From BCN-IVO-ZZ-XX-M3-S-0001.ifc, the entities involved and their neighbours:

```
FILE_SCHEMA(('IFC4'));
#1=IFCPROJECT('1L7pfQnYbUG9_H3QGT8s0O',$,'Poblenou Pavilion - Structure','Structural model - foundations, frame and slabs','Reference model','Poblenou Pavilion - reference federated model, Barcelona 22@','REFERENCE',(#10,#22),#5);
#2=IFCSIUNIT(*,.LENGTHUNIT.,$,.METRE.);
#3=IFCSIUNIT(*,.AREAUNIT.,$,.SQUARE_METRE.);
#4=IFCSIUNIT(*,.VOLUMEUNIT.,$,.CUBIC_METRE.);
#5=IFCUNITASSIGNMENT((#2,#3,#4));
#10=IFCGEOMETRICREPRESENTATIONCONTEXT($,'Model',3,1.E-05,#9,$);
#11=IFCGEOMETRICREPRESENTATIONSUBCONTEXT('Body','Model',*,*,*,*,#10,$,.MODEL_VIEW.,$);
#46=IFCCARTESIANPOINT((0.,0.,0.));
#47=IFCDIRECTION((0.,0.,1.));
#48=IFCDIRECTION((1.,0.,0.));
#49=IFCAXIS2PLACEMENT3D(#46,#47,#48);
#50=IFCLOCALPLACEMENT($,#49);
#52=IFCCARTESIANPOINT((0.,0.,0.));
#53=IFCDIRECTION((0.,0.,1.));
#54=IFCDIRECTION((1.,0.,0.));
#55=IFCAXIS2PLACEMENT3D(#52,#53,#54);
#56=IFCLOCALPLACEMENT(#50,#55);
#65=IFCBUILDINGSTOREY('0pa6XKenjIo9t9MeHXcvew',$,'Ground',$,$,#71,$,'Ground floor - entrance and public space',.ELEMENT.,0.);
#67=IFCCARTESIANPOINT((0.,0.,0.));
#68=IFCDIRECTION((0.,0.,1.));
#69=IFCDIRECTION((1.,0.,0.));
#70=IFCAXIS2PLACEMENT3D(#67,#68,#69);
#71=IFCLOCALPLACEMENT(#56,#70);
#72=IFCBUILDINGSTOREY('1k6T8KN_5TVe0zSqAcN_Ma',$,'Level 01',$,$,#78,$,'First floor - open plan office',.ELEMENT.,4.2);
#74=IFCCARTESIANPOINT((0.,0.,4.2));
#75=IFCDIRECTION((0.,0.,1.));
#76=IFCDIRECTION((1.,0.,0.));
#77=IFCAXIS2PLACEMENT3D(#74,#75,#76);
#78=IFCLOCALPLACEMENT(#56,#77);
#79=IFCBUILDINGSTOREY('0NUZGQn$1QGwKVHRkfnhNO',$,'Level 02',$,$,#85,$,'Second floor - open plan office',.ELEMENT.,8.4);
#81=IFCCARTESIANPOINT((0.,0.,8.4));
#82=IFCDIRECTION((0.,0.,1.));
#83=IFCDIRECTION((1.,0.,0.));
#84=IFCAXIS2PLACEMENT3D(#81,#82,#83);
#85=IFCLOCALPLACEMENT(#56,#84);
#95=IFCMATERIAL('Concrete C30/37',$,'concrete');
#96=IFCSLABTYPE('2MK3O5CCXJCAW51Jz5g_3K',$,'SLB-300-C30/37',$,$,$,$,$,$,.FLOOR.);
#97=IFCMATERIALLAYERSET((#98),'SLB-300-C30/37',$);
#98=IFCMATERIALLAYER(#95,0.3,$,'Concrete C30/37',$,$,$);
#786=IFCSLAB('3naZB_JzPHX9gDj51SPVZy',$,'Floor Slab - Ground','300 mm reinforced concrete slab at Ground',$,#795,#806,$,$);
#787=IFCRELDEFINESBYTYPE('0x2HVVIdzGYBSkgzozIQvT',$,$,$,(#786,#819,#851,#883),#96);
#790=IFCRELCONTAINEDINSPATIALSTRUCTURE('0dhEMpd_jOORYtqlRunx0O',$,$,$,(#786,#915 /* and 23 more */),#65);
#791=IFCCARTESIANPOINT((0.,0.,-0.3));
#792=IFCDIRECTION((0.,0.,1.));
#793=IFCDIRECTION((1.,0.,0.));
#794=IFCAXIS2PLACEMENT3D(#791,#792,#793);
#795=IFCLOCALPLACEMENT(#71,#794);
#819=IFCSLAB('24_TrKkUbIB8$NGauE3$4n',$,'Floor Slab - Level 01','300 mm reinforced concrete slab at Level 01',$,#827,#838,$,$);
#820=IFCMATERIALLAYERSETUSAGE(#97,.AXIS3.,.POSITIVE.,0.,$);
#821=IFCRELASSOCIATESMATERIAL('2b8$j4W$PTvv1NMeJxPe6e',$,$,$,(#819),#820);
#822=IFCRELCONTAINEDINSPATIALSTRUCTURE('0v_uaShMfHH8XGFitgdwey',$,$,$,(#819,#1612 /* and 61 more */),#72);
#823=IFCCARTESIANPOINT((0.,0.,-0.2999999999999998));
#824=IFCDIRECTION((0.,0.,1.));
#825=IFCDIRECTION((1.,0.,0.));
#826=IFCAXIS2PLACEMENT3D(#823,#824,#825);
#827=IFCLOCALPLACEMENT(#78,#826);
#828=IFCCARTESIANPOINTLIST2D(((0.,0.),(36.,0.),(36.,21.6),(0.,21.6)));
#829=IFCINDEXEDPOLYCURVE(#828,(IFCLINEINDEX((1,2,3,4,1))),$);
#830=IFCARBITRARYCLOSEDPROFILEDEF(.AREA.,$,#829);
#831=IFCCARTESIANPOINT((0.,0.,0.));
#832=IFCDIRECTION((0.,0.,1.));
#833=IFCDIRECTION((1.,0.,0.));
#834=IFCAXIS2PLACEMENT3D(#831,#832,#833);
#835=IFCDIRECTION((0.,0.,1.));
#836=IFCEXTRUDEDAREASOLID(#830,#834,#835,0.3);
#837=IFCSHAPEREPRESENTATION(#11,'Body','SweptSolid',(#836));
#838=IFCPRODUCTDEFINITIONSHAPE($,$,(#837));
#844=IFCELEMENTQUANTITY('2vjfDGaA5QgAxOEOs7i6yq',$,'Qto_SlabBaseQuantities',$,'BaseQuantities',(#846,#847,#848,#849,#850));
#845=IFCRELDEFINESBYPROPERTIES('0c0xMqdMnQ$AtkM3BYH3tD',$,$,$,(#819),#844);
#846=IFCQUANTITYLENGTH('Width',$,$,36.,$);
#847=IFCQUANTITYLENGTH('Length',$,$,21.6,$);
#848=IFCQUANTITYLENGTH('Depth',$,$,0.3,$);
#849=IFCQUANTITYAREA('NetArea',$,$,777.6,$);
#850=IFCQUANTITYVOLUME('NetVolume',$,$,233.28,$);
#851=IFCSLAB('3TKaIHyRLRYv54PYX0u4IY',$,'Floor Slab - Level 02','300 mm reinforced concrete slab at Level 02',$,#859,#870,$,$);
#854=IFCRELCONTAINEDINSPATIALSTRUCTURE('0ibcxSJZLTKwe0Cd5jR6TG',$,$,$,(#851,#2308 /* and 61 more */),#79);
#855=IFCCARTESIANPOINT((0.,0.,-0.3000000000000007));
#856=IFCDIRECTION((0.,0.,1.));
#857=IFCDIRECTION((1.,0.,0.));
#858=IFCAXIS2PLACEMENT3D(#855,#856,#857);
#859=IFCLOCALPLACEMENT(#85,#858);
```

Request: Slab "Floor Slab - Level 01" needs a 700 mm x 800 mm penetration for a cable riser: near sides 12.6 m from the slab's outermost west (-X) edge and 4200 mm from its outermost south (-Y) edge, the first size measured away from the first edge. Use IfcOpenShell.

```python
import numpy as np
import ifcopenshell
import ifcopenshell.api.feature
import ifcopenshell.api.geometry
import ifcopenshell.api.pset
import ifcopenshell.api.root
import ifcopenshell.geom
import ifcopenshell.util.element
import ifcopenshell.util.placement
import ifcopenshell.util.representation
import ifcopenshell.util.shape
import ifcopenshell.util.unit

model = ifcopenshell.open("BCN-IVO-ZZ-XX-M3-S-0001.ifc")
unit_scale = ifcopenshell.util.unit.calculate_unit_scale(model)
area_scale = ifcopenshell.util.unit.calculate_unit_scale(model, "AREAUNIT")
volume_scale = ifcopenshell.util.unit.calculate_unit_scale(model, "VOLUMEUNIT")
settings = ifcopenshell.geom.settings()


def volume(element):
    """Net volume in cubic metres, openings subtracted."""
    shape = ifcopenshell.geom.create_shape(settings, element)
    return ifcopenshell.util.shape.get_volume(shape.geometry)


slab = model.by_guid("24_TrKkUbIB8$NGauE3$4n")
before = volume(slab)

# Extent in the slab's own axes, in metres. The edges named are its -X and -Y sides.
slab_shape = ifcopenshell.geom.create_shape(settings, slab)
vertices = ifcopenshell.util.shape.get_vertices(slab_shape.geometry)
x_min, y_min, bottom = vertices.min(axis=0)
top = vertices[:, 2].max()

opening = ifcopenshell.api.root.create_entity(model, ifc_class="IfcOpeningElement", name="Cable riser opening", predefined_type="OPENING")
context = ifcopenshell.util.representation.get_context(model, "Model", "Body", "MODEL_VIEW")
width, depth = 0.7, 0.8
outline = [(0.0, 0.0), (width, 0.0), (width, depth), (0.0, depth), (0.0, 0.0)]
# Overshoot both faces by 50 mm so the cut is clean.
shape = ifcopenshell.api.geometry.add_slab_representation(
    model, context=context, depth=top - bottom + 0.1, polyline=outline
)
ifcopenshell.api.geometry.assign_representation(model, product=opening, representation=shape)

matrix = ifcopenshell.util.placement.get_local_placement(slab.ObjectPlacement)
matrix[:, 3] = matrix @ np.append(np.array([x_min + 12.6, y_min + 4.2, bottom - 0.05]) / unit_scale, 1.0)
ifcopenshell.api.geometry.edit_object_placement(model, product=opening, matrix=matrix, is_si=False)
ifcopenshell.api.feature.add_feature(model, feature=opening, element=slab)

after = volume(slab)

# Update the slab's stored quantities.
qto = model.by_id(ifcopenshell.util.element.get_pset(slab, "Qto_SlabBaseQuantities", should_inherit=False)["id"])
ifcopenshell.api.pset.edit_qto(model, qto=qto, properties={
    "NetArea": after / (top - bottom) / area_scale,
    "NetVolume": after / volume_scale,
})

print(f"slab volume {before:.3f} -> {after:.3f} m3")

model.write("BCN-IVO-ZZ-XX-M3-S-0001_v2.ifc")
```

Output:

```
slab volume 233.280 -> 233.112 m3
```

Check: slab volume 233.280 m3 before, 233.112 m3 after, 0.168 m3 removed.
